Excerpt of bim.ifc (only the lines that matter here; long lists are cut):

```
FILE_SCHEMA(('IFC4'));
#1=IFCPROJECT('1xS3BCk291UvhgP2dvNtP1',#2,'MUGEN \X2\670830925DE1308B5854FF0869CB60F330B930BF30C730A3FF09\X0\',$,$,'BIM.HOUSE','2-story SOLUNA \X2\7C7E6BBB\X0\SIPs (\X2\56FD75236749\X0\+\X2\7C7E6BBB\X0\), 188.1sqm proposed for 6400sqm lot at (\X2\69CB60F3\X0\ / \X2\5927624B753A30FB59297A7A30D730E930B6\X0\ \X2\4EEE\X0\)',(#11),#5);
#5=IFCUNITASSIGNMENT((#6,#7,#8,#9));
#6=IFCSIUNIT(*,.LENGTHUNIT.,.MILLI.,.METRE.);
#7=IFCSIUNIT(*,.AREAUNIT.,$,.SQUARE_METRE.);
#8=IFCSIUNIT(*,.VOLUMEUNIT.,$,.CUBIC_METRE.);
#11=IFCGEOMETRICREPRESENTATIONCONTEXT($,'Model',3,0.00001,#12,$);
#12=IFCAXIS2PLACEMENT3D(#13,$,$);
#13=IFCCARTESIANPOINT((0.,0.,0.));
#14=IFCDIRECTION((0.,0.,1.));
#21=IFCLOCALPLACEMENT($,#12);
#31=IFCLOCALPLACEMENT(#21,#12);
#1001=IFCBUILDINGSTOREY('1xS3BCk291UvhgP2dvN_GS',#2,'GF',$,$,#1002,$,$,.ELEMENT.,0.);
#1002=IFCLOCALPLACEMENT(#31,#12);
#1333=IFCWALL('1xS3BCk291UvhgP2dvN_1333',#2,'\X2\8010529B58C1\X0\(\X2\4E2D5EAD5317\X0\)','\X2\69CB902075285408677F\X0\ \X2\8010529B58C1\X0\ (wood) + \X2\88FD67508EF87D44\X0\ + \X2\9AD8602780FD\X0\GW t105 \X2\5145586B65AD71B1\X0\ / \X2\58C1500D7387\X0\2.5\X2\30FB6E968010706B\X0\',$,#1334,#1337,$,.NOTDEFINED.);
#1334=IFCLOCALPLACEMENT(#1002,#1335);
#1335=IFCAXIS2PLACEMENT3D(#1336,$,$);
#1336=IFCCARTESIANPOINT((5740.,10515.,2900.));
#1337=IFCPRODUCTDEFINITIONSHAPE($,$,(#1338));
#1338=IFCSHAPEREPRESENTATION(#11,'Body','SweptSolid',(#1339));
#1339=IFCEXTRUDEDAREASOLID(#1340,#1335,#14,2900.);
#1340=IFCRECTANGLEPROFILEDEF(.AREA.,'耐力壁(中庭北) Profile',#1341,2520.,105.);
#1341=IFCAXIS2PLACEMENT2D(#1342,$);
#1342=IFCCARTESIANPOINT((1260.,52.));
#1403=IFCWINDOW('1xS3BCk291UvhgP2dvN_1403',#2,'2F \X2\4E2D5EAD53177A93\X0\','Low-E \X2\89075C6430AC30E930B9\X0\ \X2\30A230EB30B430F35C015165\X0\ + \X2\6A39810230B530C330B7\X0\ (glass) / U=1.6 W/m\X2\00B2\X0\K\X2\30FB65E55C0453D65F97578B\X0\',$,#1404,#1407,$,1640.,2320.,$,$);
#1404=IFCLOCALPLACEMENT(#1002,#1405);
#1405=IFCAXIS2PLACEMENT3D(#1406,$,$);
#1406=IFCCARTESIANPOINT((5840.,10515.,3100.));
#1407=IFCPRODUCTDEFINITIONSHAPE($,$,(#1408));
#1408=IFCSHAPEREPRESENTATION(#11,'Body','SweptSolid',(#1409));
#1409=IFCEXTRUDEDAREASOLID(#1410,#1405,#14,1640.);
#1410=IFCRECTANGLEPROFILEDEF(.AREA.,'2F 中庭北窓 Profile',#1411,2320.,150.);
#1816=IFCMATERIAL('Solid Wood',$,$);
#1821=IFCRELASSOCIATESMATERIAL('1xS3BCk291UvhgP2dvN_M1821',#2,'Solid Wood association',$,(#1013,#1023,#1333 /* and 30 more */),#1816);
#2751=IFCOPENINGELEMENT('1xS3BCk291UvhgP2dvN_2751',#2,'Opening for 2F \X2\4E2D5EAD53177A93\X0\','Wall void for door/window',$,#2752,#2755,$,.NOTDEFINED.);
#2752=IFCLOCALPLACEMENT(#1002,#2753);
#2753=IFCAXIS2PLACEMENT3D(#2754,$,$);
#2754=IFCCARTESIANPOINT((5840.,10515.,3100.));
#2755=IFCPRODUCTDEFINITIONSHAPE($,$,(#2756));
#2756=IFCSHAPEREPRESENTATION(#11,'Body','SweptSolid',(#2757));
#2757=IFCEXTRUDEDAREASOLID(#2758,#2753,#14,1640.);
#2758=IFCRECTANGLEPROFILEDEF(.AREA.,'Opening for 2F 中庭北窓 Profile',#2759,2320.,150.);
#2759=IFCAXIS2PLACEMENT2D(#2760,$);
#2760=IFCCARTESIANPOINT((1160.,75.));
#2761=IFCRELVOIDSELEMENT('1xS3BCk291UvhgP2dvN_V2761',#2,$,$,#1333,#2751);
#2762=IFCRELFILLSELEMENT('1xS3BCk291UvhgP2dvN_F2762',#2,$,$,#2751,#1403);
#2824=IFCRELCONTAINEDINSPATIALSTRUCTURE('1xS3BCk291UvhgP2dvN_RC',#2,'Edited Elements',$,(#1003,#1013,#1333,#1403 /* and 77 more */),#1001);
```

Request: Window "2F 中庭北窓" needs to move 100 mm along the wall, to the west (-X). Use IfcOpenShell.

```python
import ifcopenshell
import ifcopenshell.api.geometry
import ifcopenshell.util.placement
import ifcopenshell.util.unit

model = ifcopenshell.open("bim.ifc")
unit_scale = ifcopenshell.util.unit.calculate_unit_scale(model)

window = model.by_guid("1xS3BCk291UvhgP2dvN_1403")
opening = window.FillsVoids[0].RelatingOpeningElement
wall = opening.VoidsElements[0].RelatingBuildingElement

wall_matrix = ifcopenshell.util.placement.get_local_placement(wall.ObjectPlacement)
shift = wall_matrix[:3, 0] * -0.1 / unit_scale
before = ifcopenshell.util.placement.get_local_placement(window.ObjectPlacement)[:3, 3].copy()

# The window is not placed relative to its opening, so move both.
for product in (opening, window):
    matrix = ifcopenshell.util.placement.get_local_placement(product.ObjectPlacement)
    matrix[:3, 3] += shift
    ifcopenshell.api.geometry.edit_object_placement(model, product=product, matrix=matrix, is_si=False)

after = ifcopenshell.util.placement.get_local_placement(window.ObjectPlacement)[:3, 3]
print("window moved by", (after - before).round(3) + 0.0)

model.write("bim_edited.ifc")
```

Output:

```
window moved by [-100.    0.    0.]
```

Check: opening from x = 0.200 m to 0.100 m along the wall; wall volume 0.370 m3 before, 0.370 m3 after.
